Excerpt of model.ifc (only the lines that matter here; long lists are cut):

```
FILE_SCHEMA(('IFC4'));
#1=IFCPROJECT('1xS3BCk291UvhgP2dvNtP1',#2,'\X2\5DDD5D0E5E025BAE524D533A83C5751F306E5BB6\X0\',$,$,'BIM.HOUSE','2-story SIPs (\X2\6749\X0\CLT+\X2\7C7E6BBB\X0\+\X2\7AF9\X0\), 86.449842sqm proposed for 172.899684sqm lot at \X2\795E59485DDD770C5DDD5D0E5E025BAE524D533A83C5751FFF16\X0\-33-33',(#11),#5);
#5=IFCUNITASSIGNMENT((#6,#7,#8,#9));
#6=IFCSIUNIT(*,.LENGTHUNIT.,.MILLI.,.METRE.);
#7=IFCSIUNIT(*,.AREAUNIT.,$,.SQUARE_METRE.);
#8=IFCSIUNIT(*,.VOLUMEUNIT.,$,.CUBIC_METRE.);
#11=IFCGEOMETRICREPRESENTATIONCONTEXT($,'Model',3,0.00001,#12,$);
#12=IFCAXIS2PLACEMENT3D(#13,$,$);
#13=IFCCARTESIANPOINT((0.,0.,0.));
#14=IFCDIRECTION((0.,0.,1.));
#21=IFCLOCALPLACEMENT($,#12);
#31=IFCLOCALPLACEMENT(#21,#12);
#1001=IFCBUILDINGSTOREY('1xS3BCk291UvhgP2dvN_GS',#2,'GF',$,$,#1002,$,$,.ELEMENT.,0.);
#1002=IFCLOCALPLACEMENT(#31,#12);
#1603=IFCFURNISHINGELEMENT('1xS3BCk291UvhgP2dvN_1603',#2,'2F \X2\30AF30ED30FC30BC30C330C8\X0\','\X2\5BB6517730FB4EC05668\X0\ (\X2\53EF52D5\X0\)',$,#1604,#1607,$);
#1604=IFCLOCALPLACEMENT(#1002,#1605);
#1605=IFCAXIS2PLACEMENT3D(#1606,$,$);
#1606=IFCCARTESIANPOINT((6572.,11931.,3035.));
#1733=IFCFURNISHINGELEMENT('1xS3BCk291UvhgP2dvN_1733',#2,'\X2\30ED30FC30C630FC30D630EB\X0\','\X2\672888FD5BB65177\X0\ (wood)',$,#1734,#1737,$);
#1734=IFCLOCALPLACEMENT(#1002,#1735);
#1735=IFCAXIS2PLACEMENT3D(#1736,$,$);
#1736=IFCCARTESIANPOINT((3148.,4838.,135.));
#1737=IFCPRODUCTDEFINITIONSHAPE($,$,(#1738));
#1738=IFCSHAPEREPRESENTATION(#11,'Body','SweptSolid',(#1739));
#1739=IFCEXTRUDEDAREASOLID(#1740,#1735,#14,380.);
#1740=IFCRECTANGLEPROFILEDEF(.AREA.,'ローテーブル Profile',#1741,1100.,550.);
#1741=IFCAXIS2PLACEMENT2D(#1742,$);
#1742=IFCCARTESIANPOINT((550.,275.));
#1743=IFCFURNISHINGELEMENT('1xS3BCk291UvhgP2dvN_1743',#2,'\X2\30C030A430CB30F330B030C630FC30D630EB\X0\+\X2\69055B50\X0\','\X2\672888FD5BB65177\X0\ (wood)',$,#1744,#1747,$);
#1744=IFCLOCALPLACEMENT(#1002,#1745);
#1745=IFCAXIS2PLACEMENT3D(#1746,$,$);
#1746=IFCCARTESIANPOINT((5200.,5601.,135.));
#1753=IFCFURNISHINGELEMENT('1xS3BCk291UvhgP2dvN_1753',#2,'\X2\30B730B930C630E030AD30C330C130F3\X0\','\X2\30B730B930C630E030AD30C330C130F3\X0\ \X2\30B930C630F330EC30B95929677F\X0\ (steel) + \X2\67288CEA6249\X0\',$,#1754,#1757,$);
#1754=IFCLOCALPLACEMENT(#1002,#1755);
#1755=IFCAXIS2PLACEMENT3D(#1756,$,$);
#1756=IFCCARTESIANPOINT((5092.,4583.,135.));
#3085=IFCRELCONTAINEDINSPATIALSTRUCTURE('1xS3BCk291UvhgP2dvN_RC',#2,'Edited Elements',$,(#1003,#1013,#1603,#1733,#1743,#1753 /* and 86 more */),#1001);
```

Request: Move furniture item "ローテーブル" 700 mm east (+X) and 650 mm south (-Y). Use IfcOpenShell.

```python
import ifcopenshell
import ifcopenshell.api.geometry
import ifcopenshell.util.placement

model = ifcopenshell.open("model.ifc")

item = model.by_id(1733)
matrix = ifcopenshell.util.placement.get_local_placement(item.ObjectPlacement)
matrix[0, 3] += 700.0
matrix[1, 3] -= 650.0
ifcopenshell.api.geometry.edit_object_placement(model, product=item, matrix=matrix, is_si=False)

print(ifcopenshell.util.placement.get_local_placement(item.ObjectPlacement).round(3) + 0.0)

model.write("model_updated.ifc")
```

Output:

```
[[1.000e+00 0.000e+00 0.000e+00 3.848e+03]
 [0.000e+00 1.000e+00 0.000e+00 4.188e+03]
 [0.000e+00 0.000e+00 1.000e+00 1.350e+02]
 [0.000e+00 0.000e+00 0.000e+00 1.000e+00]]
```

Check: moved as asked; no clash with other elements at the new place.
